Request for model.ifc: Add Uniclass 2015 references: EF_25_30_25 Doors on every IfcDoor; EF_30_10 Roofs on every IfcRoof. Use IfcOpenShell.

First a look at what the model holds.

```python
import ifcopenshell

model = ifcopenshell.open("model.ifc")
print(model.schema)
print("classifications:", [c.Name for c in model.by_type("IfcClassification")])
for ifc_class in ("IfcDoor", "IfcRoof", "IfcStair", "IfcWall", "IfcWindow"):
    print(ifc_class, len(model.by_type(ifc_class)))
```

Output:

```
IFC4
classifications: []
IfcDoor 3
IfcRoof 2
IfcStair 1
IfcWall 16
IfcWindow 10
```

```python
import ifcopenshell
import ifcopenshell.api.classification

model = ifcopenshell.open("model.ifc")

system = ifcopenshell.api.classification.add_classification(model, classification="Uniclass 2015")

codes = {
    "IfcDoor": ("EF_25_30_25", "Doors"),
    "IfcRoof": ("EF_30_10", "Roofs"),
}
for ifc_class, (code, name) in codes.items():
    products = model.by_type(ifc_class)
    ifcopenshell.api.classification.add_reference(
        model, products=products, classification=system, identification=code, name=name
    )
    print(code, len(products))

model.write("model_edited.ifc")
```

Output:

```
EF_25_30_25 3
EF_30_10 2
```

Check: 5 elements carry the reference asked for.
